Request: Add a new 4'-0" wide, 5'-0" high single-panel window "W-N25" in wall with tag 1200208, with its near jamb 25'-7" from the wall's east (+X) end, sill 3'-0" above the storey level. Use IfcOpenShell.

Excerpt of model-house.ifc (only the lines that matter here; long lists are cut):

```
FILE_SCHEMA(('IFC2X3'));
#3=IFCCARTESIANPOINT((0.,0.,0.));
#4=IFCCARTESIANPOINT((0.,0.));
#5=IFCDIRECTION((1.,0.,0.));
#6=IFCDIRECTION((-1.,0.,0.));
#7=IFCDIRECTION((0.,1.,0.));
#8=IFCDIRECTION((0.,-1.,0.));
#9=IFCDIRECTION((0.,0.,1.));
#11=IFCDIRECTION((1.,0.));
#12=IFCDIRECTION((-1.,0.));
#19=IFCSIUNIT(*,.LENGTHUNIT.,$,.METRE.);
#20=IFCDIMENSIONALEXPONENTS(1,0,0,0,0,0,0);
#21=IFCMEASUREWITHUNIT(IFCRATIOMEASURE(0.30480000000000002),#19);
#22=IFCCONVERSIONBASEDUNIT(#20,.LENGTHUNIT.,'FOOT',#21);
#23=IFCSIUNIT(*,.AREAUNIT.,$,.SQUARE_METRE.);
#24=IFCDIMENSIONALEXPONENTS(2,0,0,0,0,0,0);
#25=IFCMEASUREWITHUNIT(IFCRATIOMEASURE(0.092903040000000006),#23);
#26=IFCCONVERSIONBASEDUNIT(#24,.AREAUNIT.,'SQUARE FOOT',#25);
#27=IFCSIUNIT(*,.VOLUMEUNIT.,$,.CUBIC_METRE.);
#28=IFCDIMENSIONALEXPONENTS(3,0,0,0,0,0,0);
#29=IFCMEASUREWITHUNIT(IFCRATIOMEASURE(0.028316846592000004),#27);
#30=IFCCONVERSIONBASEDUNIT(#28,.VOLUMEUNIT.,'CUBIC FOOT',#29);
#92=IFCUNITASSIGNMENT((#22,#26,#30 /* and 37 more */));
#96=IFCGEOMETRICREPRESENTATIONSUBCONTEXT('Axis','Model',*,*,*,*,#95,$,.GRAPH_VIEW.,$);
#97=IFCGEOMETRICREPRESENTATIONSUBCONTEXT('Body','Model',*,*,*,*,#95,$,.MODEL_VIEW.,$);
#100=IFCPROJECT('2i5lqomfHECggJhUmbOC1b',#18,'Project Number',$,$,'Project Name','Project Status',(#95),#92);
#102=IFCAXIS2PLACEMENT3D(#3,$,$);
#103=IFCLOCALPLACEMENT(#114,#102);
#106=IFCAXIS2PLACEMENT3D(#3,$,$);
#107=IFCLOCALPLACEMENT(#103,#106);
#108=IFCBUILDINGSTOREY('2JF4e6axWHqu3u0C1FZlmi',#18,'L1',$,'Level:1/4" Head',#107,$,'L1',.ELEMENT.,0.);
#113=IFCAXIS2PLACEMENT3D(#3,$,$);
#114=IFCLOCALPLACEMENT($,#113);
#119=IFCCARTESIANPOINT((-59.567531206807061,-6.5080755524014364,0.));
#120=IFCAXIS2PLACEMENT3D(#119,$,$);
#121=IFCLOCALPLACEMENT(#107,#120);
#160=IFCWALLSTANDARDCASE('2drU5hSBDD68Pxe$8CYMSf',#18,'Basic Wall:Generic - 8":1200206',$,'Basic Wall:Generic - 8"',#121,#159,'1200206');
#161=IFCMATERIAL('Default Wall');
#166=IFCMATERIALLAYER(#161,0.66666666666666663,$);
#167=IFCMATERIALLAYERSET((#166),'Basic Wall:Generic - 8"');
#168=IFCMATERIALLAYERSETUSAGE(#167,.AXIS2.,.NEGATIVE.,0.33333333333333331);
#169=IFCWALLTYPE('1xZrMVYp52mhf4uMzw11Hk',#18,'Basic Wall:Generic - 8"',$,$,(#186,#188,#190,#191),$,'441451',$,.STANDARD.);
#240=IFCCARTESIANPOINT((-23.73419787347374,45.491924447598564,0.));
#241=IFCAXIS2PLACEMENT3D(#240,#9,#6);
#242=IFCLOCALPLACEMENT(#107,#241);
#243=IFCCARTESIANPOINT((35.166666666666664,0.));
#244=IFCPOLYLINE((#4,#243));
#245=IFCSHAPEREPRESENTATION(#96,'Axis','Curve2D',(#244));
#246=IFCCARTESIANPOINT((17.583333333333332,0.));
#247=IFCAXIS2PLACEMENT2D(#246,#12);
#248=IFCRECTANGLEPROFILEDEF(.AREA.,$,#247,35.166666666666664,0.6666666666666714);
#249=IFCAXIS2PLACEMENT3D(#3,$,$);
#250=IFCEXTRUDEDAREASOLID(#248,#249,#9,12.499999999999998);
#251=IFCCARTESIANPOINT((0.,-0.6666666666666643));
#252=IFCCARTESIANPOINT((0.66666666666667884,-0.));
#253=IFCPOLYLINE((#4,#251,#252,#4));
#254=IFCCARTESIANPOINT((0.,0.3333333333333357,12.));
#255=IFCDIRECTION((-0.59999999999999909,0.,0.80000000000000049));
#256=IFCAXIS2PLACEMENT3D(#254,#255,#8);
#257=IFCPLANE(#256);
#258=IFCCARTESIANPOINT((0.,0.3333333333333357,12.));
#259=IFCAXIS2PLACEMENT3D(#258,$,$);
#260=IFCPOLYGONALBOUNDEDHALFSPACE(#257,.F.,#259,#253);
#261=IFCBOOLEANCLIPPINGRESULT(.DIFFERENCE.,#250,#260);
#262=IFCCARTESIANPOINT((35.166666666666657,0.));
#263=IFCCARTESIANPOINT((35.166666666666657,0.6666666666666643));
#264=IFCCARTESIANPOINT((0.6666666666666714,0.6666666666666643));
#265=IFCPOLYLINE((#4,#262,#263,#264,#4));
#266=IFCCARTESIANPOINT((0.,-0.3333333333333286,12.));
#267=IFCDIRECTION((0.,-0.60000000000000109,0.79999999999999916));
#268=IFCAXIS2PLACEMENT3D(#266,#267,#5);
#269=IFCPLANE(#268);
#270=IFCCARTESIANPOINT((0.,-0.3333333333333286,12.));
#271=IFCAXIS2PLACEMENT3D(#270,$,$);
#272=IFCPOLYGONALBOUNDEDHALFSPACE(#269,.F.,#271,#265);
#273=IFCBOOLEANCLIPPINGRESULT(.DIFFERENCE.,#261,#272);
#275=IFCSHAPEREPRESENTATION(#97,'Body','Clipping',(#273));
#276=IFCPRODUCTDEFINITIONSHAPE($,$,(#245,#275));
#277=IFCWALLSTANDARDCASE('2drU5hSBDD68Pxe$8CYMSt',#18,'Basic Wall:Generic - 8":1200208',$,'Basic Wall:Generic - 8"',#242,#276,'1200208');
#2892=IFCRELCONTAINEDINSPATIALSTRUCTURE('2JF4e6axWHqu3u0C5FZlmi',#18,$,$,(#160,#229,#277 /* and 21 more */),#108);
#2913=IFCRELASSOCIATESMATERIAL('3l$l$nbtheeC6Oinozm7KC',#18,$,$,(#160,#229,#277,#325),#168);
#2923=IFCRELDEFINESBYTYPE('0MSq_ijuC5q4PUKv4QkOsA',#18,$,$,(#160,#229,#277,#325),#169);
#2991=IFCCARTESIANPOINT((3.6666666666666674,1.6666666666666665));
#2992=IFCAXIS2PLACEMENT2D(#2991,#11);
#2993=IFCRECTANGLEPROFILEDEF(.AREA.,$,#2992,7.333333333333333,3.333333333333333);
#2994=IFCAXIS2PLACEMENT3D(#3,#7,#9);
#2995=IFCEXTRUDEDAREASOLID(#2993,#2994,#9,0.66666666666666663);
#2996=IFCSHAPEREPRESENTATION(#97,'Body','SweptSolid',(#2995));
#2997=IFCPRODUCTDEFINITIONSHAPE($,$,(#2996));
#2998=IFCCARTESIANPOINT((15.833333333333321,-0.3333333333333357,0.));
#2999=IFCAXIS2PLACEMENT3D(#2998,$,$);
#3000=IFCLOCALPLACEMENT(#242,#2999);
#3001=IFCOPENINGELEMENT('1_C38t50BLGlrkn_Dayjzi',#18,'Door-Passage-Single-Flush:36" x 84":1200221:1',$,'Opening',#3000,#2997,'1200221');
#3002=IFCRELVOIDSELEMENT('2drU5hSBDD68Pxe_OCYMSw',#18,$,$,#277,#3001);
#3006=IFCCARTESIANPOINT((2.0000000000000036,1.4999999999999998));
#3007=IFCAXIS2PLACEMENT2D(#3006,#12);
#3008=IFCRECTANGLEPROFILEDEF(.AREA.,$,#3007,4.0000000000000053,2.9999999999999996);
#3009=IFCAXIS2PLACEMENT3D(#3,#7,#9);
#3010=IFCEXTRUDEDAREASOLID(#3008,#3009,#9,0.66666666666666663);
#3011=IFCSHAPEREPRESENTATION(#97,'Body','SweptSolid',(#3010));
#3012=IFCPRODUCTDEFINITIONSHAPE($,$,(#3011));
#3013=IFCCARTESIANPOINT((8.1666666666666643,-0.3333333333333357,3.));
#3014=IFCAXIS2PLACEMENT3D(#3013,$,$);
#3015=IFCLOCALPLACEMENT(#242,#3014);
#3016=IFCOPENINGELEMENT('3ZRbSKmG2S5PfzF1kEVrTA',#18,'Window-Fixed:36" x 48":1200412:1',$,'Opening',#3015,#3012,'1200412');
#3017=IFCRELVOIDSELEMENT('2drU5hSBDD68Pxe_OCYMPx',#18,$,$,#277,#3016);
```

```python
import numpy as np
import ifcopenshell
import ifcopenshell.api.feature
import ifcopenshell.api.geometry
import ifcopenshell.api.root
import ifcopenshell.api.spatial
import ifcopenshell.api.type
import ifcopenshell.geom
import ifcopenshell.util.element
import ifcopenshell.util.placement
import ifcopenshell.util.representation
import ifcopenshell.util.shape
import ifcopenshell.util.unit

model = ifcopenshell.open("model-house.ifc")
unit_scale = ifcopenshell.util.unit.calculate_unit_scale(model)
settings = ifcopenshell.geom.settings()


def volume(element):
    """Net volume in cubic metres, openings subtracted."""
    shape = ifcopenshell.geom.create_shape(settings, element)
    return ifcopenshell.util.shape.get_volume(shape.geometry)


wall = model.by_guid("2drU5hSBDD68Pxe$8CYMSt")
storey = ifcopenshell.util.element.get_container(wall, ifc_class="IfcBuildingStorey")
context = ifcopenshell.util.representation.get_context(model, "Model", "Body", "MODEL_VIEW")
before = volume(wall)

width, height, from_end, sill = 1.2192, 1.524, 7.7978, 0.9144  # metres

# The wall runs along its own X axis, and the end named is its -X end.
wall_shape = ifcopenshell.geom.create_shape(settings, wall)
x, y, z = ifcopenshell.util.shape.get_vertices(wall_shape.geometry).T
start = x.min() + from_end
face, thickness = float(y.min()), float(y.max() - y.min())
wall_matrix = ifcopenshell.util.placement.get_local_placement(wall.ObjectPlacement)
level = ifcopenshell.util.placement.get_local_placement(storey.ObjectPlacement)[2, 3]


def in_wall(x, y):
    """Placement at x, y metres in the wall's axes, at sill height."""
    matrix = wall_matrix.copy()
    matrix[:, 3] = wall_matrix @ np.array([x / unit_scale, y / unit_scale, 0.0, 1.0])
    matrix[2, 3] = level + sill / unit_scale
    return matrix


# Opening: a box that overshoots both wall faces by 50 mm.
opening = ifcopenshell.api.root.create_entity(model, ifc_class="IfcOpeningElement")
box = ifcopenshell.api.geometry.add_wall_representation(
    model, context=context, length=width, height=height, thickness=thickness + 0.1
)
ifcopenshell.api.geometry.assign_representation(model, product=opening, representation=box)
ifcopenshell.api.geometry.edit_object_placement(model, product=opening, matrix=in_wall(start, face - 0.05), is_si=False)
ifcopenshell.api.feature.add_feature(model, feature=opening, element=wall)

window = ifcopenshell.api.root.create_entity(model, ifc_class="IfcWindow", name="W-N25")
window.OverallWidth, window.OverallHeight = width / unit_scale, height / unit_scale
body = ifcopenshell.api.geometry.add_window_representation(
    model,
    context=context,
    overall_width=window.OverallWidth,
    overall_height=window.OverallHeight,
    partition_type="SINGLE_PANEL",
)
ifcopenshell.api.geometry.assign_representation(model, product=window, representation=body)
ifcopenshell.api.spatial.assign_container(model, products=[window], relating_structure=storey)
fills = ifcopenshell.api.feature.add_filling(model, opening=opening, element=window)
fills.OwnerHistory = window.OwnerHistory  # required in IFC2X3

# IFC2X3 keeps the operation on the window style.
style = ifcopenshell.api.root.create_entity(model, ifc_class="IfcWindowStyle", name="W-N25")
style.OperationType, style.ConstructionType = "SINGLE_PANEL", "NOTDEFINED"
style.ParameterTakesPrecedence = style.Sizeable = False
ifcopenshell.api.type.assign_type(model, related_objects=[window], relating_type=style)

# Centre the window in the wall's thickness.
ifcopenshell.api.geometry.edit_object_placement(model, product=window, matrix=in_wall(start, face), is_si=False)
window_shape = ifcopenshell.geom.create_shape(settings, window)
depth = ifcopenshell.util.shape.get_vertices(window_shape.geometry)[:, 1]
offset = face + thickness / 2 - (depth.min() + depth.max()) / 2
ifcopenshell.api.geometry.edit_object_placement(model, product=window, matrix=in_wall(start, offset), is_si=False)

after = volume(wall)

print(f"wall volume {before:.3f} -> {after:.3f} m3")

model.write("model-house_edited.ifc")
```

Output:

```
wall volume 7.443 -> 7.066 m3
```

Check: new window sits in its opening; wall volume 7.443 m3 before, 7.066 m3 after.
